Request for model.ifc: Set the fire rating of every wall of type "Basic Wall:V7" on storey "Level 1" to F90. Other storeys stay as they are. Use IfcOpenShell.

First a look at what the model holds.

```python
import ifcopenshell
import ifcopenshell.util.element

model = ifcopenshell.open("model.ifc")
print(model.schema)
storey = next(s for s in model.by_type("IfcBuildingStorey") if s.Name == "Level 1")
walls = [e for e in ifcopenshell.util.element.get_decomposition(storey) if e.is_a("IfcWall")]
seen = {}
for e in walls:
    element_type = ifcopenshell.util.element.get_type(e)
    key = (element_type.Name if element_type != e and element_type else None, ifcopenshell.util.element.get_pset(e, "Pset_WallCommon", "FireRating"))
    seen[key] = seen.get(key, 0) + 1
for (name, value), count in sorted(seen.items(), key=str):
    print(count, "x", name, "|", value)
```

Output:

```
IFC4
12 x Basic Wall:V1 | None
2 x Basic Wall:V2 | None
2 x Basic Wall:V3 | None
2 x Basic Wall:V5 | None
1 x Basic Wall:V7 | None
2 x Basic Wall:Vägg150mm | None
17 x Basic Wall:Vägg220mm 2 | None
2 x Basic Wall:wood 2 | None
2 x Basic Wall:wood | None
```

```python
import ifcopenshell
import ifcopenshell.api.pset
import ifcopenshell.util.element

model = ifcopenshell.open("model.ifc")

storey = next(s for s in model.by_type("IfcBuildingStorey") if s.Name == "Level 1")
walls = [e for e in ifcopenshell.util.element.get_decomposition(storey) if e.is_a("IfcWall")]

count = 0
for e in walls:
    element_type = ifcopenshell.util.element.get_type(e)
    if element_type in (None, e) or element_type.Name != "Basic Wall:V7":
        continue
    # add_pset returns the element's existing set when there is one.
    pset = ifcopenshell.api.pset.add_pset(model, product=e, name="Pset_WallCommon")
    ifcopenshell.api.pset.edit_pset(model, pset=pset, properties={"FireRating": "F90"})
    count += 1

print(count, "walls updated")

model.write("model_updated.ifc")
```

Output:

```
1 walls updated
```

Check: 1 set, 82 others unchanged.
